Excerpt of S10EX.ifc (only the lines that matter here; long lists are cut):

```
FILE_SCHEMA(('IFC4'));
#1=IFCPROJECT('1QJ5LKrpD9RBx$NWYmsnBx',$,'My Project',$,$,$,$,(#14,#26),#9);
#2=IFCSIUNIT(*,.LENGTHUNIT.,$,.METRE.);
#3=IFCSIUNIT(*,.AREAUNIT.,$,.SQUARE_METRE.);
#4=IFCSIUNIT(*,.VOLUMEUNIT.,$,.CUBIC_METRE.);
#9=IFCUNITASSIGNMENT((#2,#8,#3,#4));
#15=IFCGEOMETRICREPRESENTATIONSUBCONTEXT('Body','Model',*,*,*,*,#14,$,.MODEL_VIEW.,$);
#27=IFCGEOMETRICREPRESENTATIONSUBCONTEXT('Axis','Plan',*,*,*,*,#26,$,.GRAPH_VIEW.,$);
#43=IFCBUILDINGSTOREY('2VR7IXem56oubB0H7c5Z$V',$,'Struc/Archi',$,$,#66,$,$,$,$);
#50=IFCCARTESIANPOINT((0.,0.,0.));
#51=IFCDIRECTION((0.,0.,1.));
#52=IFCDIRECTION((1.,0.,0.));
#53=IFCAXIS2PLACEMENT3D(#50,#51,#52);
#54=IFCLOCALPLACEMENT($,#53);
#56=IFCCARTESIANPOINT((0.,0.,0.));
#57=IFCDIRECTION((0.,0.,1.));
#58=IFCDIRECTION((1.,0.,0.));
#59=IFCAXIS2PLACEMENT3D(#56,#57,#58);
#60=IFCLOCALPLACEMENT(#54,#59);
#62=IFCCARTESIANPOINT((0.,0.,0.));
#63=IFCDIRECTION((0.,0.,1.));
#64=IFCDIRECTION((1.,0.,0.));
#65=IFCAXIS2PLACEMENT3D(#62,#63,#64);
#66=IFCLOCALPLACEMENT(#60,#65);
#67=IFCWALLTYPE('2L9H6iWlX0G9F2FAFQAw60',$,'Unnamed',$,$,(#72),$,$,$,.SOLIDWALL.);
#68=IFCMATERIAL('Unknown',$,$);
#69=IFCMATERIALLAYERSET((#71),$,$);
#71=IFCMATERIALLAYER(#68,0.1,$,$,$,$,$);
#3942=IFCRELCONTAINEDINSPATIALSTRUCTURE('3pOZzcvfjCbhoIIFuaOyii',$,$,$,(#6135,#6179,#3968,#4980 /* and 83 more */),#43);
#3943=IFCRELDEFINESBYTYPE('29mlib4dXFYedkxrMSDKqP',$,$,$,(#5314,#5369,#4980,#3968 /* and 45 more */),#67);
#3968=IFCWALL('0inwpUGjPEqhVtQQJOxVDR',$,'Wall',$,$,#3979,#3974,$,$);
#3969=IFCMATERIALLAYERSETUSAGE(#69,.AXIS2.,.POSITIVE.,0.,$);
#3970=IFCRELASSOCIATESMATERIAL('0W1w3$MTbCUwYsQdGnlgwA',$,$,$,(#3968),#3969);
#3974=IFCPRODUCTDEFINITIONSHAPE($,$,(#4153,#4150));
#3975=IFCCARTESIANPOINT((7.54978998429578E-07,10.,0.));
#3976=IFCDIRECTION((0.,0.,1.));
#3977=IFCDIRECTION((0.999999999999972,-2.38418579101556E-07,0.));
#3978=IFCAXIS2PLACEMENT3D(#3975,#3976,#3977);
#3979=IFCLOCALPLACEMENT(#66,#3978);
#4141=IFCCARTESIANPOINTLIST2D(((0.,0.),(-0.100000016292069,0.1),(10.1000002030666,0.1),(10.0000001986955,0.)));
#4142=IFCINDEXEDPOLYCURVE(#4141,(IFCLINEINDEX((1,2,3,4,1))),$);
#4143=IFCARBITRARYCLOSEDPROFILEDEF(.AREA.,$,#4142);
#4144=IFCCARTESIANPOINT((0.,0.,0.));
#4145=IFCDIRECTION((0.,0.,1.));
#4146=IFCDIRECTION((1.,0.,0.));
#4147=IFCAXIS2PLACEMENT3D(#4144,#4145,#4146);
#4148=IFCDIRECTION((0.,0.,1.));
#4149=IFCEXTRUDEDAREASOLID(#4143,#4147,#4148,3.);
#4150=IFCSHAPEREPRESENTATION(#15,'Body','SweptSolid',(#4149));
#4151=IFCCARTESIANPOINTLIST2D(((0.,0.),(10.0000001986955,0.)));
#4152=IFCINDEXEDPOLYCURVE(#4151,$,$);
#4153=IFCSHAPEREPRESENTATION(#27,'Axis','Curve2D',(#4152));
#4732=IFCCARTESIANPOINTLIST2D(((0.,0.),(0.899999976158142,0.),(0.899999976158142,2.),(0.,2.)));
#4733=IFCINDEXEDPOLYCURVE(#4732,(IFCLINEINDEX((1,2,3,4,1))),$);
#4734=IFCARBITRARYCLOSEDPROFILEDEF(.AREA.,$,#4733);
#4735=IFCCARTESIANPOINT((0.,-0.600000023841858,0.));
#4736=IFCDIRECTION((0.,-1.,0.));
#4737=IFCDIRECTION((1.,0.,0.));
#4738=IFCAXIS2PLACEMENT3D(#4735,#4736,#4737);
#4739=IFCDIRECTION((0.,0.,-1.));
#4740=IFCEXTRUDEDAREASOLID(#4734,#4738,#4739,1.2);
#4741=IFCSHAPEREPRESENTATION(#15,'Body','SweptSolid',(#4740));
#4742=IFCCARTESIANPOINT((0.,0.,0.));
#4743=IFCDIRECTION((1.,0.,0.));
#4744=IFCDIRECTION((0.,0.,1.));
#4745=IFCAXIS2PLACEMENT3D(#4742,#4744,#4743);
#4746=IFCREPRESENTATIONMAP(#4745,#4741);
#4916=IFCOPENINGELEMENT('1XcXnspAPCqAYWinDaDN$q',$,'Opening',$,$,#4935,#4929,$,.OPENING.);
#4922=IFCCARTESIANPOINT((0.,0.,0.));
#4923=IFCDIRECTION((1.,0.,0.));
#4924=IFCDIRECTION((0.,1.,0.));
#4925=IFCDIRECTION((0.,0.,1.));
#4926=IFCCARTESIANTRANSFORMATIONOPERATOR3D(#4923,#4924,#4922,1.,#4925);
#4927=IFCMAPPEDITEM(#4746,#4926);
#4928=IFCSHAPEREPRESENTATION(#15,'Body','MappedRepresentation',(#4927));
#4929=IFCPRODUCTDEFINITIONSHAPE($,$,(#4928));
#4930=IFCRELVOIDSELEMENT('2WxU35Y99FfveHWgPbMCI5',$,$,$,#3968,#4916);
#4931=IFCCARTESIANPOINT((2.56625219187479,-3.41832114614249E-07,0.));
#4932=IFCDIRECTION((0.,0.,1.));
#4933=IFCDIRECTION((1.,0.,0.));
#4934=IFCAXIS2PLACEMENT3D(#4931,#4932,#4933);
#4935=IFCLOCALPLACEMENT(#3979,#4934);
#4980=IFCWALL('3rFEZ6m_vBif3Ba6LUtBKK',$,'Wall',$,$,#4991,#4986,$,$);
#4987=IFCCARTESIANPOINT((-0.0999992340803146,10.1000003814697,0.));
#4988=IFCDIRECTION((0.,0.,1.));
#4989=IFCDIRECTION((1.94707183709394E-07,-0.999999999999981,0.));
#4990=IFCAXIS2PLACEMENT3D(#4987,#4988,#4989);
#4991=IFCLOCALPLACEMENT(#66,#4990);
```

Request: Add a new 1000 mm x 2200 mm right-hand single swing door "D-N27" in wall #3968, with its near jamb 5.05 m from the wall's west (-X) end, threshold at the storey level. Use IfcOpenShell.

```python
import numpy as np
import ifcopenshell
import ifcopenshell.api.feature
import ifcopenshell.api.geometry
import ifcopenshell.api.root
import ifcopenshell.api.spatial
import ifcopenshell.geom
import ifcopenshell.util.element
import ifcopenshell.util.placement
import ifcopenshell.util.representation
import ifcopenshell.util.shape
import ifcopenshell.util.unit

model = ifcopenshell.open("S10EX.ifc")
unit_scale = ifcopenshell.util.unit.calculate_unit_scale(model)
settings = ifcopenshell.geom.settings()


def volume(element):
    """Net volume in cubic metres, openings subtracted."""
    shape = ifcopenshell.geom.create_shape(settings, element)
    return ifcopenshell.util.shape.get_volume(shape.geometry)


wall = model.by_guid("0inwpUGjPEqhVtQQJOxVDR")
storey = ifcopenshell.util.element.get_container(wall, ifc_class="IfcBuildingStorey")
context = ifcopenshell.util.representation.get_context(model, "Model", "Body", "MODEL_VIEW")
before = volume(wall)

width, height, from_end, sill = 1, 2.2, 5.05, 0.0  # metres

# The wall runs along its own X axis, and the end named is its -X end.
wall_shape = ifcopenshell.geom.create_shape(settings, wall)
x, y, z = ifcopenshell.util.shape.get_vertices(wall_shape.geometry).T
start = x.min() + from_end
face, thickness = float(y.min()), float(y.max() - y.min())
wall_matrix = ifcopenshell.util.placement.get_local_placement(wall.ObjectPlacement)
level = ifcopenshell.util.placement.get_local_placement(storey.ObjectPlacement)[2, 3]


def in_wall(x, y):
    """Placement at x, y metres in the wall's axes, at sill height."""
    matrix = wall_matrix.copy()
    matrix[:, 3] = wall_matrix @ np.array([x / unit_scale, y / unit_scale, 0.0, 1.0])
    matrix[2, 3] = level + sill / unit_scale
    return matrix


# Opening: a box that overshoots both wall faces by 50 mm.
opening = ifcopenshell.api.root.create_entity(model, ifc_class="IfcOpeningElement", predefined_type="OPENING")
box = ifcopenshell.api.geometry.add_wall_representation(
    model, context=context, length=width, height=height, thickness=thickness + 0.1
)
ifcopenshell.api.geometry.assign_representation(model, product=opening, representation=box)
ifcopenshell.api.geometry.edit_object_placement(model, product=opening, matrix=in_wall(start, face - 0.05), is_si=False)
ifcopenshell.api.feature.add_feature(model, feature=opening, element=wall)

door = ifcopenshell.api.root.create_entity(model, ifc_class="IfcDoor", name="D-N27", predefined_type="DOOR")
door.OverallWidth, door.OverallHeight = width / unit_scale, height / unit_scale
door.OperationType = "SINGLE_SWING_RIGHT"
body = ifcopenshell.api.geometry.add_door_representation(
    model,
    context=context,
    overall_width=door.OverallWidth,
    overall_height=door.OverallHeight,
    operation_type="SINGLE_SWING_RIGHT",
    lining_properties={"LiningDepth": thickness / unit_scale, "ThresholdDepth": thickness / unit_scale},
)
ifcopenshell.api.geometry.assign_representation(model, product=door, representation=body)
ifcopenshell.api.spatial.assign_container(model, products=[door], relating_structure=storey)
ifcopenshell.api.feature.add_filling(model, opening=opening, element=door)

# The lining spans the wall, so the door starts at the wall face.
ifcopenshell.api.geometry.edit_object_placement(model, product=door, matrix=in_wall(start, face), is_si=False)

after = volume(wall)

print(f"wall volume {before:.3f} -> {after:.3f} m3")

model.write("S10EX-out.ifc")
```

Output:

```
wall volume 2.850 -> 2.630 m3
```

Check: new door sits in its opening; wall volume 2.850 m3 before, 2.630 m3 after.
